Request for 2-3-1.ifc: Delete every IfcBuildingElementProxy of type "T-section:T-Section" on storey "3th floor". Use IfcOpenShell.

First a look at what the model holds.

```python
import ifcopenshell
import ifcopenshell.util.element

model = ifcopenshell.open("2-3-1.ifc")
print(model.schema)
storey = next(s for s in model.by_type("IfcBuildingStorey") if s.Name == "3th floor")
proxies = [e for e in ifcopenshell.util.element.get_decomposition(storey) if e.is_a("IfcBuildingElementProxy")]
seen = {}
for e in proxies:
    element_type = ifcopenshell.util.element.get_type(e)
    name = element_type.Name if element_type not in (None, e) else None
    seen[name] = seen.get(name, 0) + 1
for name, count in sorted(seen.items(), key=str):
    print(count, "x", name)
```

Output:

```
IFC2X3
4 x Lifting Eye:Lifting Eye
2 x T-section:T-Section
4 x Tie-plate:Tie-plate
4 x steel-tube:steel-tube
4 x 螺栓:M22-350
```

```python
import ifcopenshell
import ifcopenshell.api.root
import ifcopenshell.util.element

model = ifcopenshell.open("2-3-1.ifc")

storey = next(s for s in model.by_type("IfcBuildingStorey") if s.Name == "3th floor")
proxies = [e for e in ifcopenshell.util.element.get_decomposition(storey) if e.is_a("IfcBuildingElementProxy")]
targets = [e for e in proxies if (t := ifcopenshell.util.element.get_type(e)) not in (None, e) and t.Name == "T-section:T-Section"]

for e in targets:
    ifcopenshell.api.root.remove_product(model, product=e)
print(len(targets), "removed")

model.write("2-3-1_edited.ifc")
```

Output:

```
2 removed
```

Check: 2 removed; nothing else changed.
